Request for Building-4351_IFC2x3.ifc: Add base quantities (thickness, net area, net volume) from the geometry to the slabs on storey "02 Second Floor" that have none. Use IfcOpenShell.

First a look at what the model holds.

```python
import ifcopenshell
import ifcopenshell.util.element
import ifcopenshell.util.unit

model = ifcopenshell.open("Building-4351_IFC2x3.ifc")
print(model.schema)
for unit_type in ("LENGTHUNIT", "AREAUNIT", "VOLUMEUNIT"):
    print(unit_type, ifcopenshell.util.unit.calculate_unit_scale(model, unit_type))
storey = next(s for s in model.by_type("IfcBuildingStorey") if s.Name == "02 Second Floor")
slabs = [e for e in ifcopenshell.util.element.get_decomposition(storey) if e.is_a("IfcSlab")]
for e in sorted(slabs, key=lambda e: e.id()):
    print(e.id(), e.is_a(), e.Name, list(ifcopenshell.util.element.get_psets(e, qtos_only=True)), sep=" | ")
```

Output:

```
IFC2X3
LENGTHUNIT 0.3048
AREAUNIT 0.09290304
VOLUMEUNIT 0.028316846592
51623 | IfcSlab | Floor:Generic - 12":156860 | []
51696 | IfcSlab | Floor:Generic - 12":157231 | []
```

```python
import ifcopenshell
import ifcopenshell.api.pset
import ifcopenshell.geom
import ifcopenshell.util.element
import ifcopenshell.util.shape
import ifcopenshell.util.unit

model = ifcopenshell.open("Building-4351_IFC2x3.ifc")
unit_scale = ifcopenshell.util.unit.calculate_unit_scale(model)
area_scale = ifcopenshell.util.unit.calculate_unit_scale(model, "AREAUNIT")
volume_scale = ifcopenshell.util.unit.calculate_unit_scale(model, "VOLUMEUNIT")
settings = ifcopenshell.geom.settings()

storey = next(s for s in model.by_type("IfcBuildingStorey") if s.Name == "02 Second Floor")
slabs = [e for e in ifcopenshell.util.element.get_decomposition(storey) if e.is_a("IfcSlab")]

for e in sorted(slabs, key=lambda e: e.id()):
    if ifcopenshell.util.element.get_psets(e, qtos_only=True, should_inherit=False):
        continue
    # Geometry comes back in metres, in the element's own axes.
    shape = ifcopenshell.geom.create_shape(settings, e)
    values = {
        "Width": ifcopenshell.util.shape.get_z(shape.geometry) / unit_scale,
        "NetArea": ifcopenshell.util.shape.get_footprint_area(shape.geometry) / area_scale,
        "NetVolume": ifcopenshell.util.shape.get_volume(shape.geometry) / volume_scale,
    }
    qto = ifcopenshell.api.pset.add_qto(model, product=e, name="BaseQuantities")
    ifcopenshell.api.pset.edit_qto(model, qto=qto, properties=values)
    print(e.id(), {k: round(v, 3) for k, v in values.items()})

model.write("Building-4351_IFC2x3_edited.ifc")
```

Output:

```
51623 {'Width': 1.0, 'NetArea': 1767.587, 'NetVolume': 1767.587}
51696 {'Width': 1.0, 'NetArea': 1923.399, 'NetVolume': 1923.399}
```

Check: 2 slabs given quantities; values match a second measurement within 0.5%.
